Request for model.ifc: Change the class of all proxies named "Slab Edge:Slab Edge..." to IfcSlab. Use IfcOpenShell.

First a look at what the model holds.

```python
import re

import ifcopenshell

model = ifcopenshell.open("model.ifc")
print(model.schema)
seen = {}
for e in model.by_type("IfcBuildingElementProxy"):
    name = re.sub(r":\d+(:\d+)?$", "", e.Name or "")  # drop the element id that some exporters append
    seen[name] = seen.get(name, 0) + 1
for name, count in sorted(seen.items()):
    print(count, "x", name)
```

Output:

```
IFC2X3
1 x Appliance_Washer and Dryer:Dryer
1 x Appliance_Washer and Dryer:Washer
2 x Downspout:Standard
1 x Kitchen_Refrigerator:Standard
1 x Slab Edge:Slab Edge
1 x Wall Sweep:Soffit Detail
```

```python
import ifcopenshell
import ifcopenshell.api.root

model = ifcopenshell.open("model.ifc")

proxies = [e.id() for e in model.by_type("IfcBuildingElementProxy") if (e.Name or "").startswith("Slab Edge:Slab Edge")]
for step_id in proxies:
    proxy = model.by_id(step_id)
    # Reclassifying a typed element also reclassifies its type and the type's other occurrences.
    if proxy.is_a("IfcBuildingElementProxy"):
        ifcopenshell.api.root.reassign_class(model, product=proxy, ifc_class="IfcSlab", predefined_type="FLOOR")

print(sum(model.by_id(i).is_a("IfcSlab") for i in proxies), "reclassified")

model.write("model_updated.ifc")
```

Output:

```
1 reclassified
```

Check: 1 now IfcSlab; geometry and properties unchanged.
